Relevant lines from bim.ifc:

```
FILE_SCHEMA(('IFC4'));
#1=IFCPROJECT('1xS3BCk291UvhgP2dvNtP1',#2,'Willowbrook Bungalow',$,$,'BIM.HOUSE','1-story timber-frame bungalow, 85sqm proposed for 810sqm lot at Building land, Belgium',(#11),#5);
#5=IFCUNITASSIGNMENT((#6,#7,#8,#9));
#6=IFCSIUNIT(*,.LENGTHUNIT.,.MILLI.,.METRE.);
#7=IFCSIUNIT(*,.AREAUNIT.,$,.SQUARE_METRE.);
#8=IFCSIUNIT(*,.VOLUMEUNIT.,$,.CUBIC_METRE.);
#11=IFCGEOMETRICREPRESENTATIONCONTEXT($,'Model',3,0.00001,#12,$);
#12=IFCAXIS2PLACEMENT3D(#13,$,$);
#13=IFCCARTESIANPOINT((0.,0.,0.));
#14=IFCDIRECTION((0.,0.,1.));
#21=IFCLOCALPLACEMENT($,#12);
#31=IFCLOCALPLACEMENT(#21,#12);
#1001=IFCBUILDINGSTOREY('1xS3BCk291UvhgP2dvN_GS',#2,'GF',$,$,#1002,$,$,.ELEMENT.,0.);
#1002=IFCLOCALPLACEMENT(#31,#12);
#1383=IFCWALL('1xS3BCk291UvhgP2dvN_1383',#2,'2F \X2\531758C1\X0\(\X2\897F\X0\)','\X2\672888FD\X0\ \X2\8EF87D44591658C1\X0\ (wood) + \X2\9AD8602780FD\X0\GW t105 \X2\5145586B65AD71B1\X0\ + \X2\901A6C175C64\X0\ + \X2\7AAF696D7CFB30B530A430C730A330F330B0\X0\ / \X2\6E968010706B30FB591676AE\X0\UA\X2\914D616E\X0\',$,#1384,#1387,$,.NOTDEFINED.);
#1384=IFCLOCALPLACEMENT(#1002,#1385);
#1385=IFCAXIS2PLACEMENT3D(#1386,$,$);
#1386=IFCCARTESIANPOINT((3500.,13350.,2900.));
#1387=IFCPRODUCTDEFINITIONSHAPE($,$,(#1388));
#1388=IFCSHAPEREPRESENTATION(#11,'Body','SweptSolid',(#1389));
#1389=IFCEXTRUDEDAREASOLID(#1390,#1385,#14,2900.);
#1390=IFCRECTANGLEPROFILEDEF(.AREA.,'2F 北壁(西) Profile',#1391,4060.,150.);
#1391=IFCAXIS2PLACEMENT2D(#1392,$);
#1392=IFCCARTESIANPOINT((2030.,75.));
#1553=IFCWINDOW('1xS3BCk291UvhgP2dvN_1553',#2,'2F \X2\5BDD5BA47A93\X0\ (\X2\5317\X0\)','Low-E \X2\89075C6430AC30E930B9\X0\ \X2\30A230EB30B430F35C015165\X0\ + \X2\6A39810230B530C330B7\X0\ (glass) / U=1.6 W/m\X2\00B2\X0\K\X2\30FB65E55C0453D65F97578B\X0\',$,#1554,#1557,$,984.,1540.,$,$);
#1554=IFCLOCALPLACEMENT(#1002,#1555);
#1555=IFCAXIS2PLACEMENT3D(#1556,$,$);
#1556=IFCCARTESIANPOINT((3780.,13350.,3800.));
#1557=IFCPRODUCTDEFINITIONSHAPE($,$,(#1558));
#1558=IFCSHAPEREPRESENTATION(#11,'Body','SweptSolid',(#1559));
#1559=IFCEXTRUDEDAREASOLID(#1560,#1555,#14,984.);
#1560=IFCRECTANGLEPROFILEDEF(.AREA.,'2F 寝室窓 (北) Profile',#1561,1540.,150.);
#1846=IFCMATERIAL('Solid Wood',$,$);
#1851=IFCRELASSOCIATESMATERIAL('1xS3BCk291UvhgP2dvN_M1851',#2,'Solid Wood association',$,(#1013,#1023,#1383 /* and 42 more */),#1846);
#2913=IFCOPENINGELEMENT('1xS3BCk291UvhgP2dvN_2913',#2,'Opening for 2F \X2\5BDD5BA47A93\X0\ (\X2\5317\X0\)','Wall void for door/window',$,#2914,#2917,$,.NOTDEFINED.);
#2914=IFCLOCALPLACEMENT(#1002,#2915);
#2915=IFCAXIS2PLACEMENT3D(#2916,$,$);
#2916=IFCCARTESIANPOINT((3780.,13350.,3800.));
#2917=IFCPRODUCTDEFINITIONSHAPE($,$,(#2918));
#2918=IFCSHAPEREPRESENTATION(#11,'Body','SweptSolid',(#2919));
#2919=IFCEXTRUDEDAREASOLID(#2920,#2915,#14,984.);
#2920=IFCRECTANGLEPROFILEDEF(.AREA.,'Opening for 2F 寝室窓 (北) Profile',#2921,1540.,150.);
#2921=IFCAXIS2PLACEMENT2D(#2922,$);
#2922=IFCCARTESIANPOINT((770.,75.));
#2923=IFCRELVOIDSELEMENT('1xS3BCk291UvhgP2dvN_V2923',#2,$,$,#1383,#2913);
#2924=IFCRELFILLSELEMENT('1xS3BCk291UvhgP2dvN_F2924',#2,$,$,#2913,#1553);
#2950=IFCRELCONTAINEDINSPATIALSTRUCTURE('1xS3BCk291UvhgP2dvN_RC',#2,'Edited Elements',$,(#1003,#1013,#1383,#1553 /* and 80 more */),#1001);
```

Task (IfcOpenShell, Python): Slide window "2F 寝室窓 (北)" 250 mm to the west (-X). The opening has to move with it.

```python
import ifcopenshell
import ifcopenshell.api.geometry
import ifcopenshell.util.placement

model = ifcopenshell.open("bim.ifc")

window = model.by_guid("1xS3BCk291UvhgP2dvN_1553")
opening = window.FillsVoids[0].RelatingOpeningElement
wall = opening.VoidsElements[0].RelatingBuildingElement

wall_matrix = ifcopenshell.util.placement.get_local_placement(wall.ObjectPlacement)
shift = wall_matrix[:3, 0] * -250.0
before = ifcopenshell.util.placement.get_local_placement(window.ObjectPlacement)[:3, 3].copy()

# The window is not placed relative to its opening, so move both.
for product in (opening, window):
    matrix = ifcopenshell.util.placement.get_local_placement(product.ObjectPlacement)
    matrix[:3, 3] += shift
    ifcopenshell.api.geometry.edit_object_placement(model, product=product, matrix=matrix, is_si=False)

after = ifcopenshell.util.placement.get_local_placement(window.ObjectPlacement)[:3, 3]
print("window moved by", (after - before).round(3) + 0.0)

model.write("bim_v2.ifc")
```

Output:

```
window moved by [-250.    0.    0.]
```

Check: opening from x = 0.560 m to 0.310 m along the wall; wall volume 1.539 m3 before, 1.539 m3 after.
